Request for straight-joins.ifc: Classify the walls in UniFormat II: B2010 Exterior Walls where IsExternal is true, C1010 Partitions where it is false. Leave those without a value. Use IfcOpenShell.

First a look at what the model holds.

```python
import ifcopenshell
import ifcopenshell.util.element

model = ifcopenshell.open("straight-joins.ifc")
print(model.schema)
print("classifications:", [c.Name for c in model.by_type("IfcClassification")])
values = [ifcopenshell.util.element.get_pset(e, "Pset_WallCommon", "IsExternal") for e in model.by_type("IfcWall")]
for value in (True, False, None):
    print("IsExternal", value, values.count(value))
```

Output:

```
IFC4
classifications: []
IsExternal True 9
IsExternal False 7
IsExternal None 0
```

```python
import ifcopenshell
import ifcopenshell.api.classification
import ifcopenshell.util.element

model = ifcopenshell.open("straight-joins.ifc")

system = ifcopenshell.api.classification.add_classification(model, classification="UniFormat II")

walls = model.by_type("IfcWall")
external = {e: ifcopenshell.util.element.get_pset(e, "Pset_WallCommon", "IsExternal") for e in walls}
for flag, code, name in ((True, "B2010", "Exterior Walls"), (False, "C1010", "Partitions")):
    products = [e for e in walls if external[e] is flag]
    ifcopenshell.api.classification.add_reference(
        model, products=products, classification=system, identification=code, name=name
    )
    print(code, len(products))

model.write("straight-joins-out.ifc")
```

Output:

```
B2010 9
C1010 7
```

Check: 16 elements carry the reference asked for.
